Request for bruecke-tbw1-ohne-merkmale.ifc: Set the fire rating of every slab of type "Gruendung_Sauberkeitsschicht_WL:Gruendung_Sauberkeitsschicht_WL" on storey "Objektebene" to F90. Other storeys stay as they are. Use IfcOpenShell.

First a look at what the model holds.

```python
import ifcopenshell
import ifcopenshell.util.element

model = ifcopenshell.open("bruecke-tbw1-ohne-merkmale.ifc")
print(model.schema)
storey = next(s for s in model.by_type("IfcBuildingStorey") if s.Name == "Objektebene")
slabs = [e for e in ifcopenshell.util.element.get_decomposition(storey) if e.is_a("IfcSlab")]
seen = {}
for e in slabs:
    element_type = ifcopenshell.util.element.get_type(e)
    key = (element_type.Name if element_type != e and element_type else None, ifcopenshell.util.element.get_pset(e, "Pset_SlabCommon", "FireRating"))
    seen[key] = seen.get(key, 0) + 1
for (name, value), count in sorted(seen.items(), key=str):
    print(count, "x", name, "|", value)
```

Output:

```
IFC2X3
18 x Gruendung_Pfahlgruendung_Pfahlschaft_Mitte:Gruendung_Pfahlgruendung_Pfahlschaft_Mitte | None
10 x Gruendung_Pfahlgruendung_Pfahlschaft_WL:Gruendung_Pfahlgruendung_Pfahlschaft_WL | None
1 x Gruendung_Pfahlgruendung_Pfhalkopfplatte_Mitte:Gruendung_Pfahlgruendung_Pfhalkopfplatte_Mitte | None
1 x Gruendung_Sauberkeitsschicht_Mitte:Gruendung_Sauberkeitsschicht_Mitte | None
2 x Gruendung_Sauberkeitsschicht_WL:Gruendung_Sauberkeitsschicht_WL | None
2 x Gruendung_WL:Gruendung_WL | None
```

```python
import ifcopenshell
import ifcopenshell.api.pset
import ifcopenshell.util.element

model = ifcopenshell.open("bruecke-tbw1-ohne-merkmale.ifc")

storey = next(s for s in model.by_type("IfcBuildingStorey") if s.Name == "Objektebene")
slabs = [e for e in ifcopenshell.util.element.get_decomposition(storey) if e.is_a("IfcSlab")]

count = 0
for e in slabs:
    element_type = ifcopenshell.util.element.get_type(e)
    if element_type in (None, e) or element_type.Name != "Gruendung_Sauberkeitsschicht_WL:Gruendung_Sauberkeitsschicht_WL":
        continue
    # add_pset returns the element's existing set when there is one.
    pset = ifcopenshell.api.pset.add_pset(model, product=e, name="Pset_SlabCommon")
    ifcopenshell.api.pset.edit_pset(model, pset=pset, properties={"FireRating": "F90"})
    count += 1

print(count, "slabs updated")

model.write("bruecke-tbw1-ohne-merkmale-out.ifc")
```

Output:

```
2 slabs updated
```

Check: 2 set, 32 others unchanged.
